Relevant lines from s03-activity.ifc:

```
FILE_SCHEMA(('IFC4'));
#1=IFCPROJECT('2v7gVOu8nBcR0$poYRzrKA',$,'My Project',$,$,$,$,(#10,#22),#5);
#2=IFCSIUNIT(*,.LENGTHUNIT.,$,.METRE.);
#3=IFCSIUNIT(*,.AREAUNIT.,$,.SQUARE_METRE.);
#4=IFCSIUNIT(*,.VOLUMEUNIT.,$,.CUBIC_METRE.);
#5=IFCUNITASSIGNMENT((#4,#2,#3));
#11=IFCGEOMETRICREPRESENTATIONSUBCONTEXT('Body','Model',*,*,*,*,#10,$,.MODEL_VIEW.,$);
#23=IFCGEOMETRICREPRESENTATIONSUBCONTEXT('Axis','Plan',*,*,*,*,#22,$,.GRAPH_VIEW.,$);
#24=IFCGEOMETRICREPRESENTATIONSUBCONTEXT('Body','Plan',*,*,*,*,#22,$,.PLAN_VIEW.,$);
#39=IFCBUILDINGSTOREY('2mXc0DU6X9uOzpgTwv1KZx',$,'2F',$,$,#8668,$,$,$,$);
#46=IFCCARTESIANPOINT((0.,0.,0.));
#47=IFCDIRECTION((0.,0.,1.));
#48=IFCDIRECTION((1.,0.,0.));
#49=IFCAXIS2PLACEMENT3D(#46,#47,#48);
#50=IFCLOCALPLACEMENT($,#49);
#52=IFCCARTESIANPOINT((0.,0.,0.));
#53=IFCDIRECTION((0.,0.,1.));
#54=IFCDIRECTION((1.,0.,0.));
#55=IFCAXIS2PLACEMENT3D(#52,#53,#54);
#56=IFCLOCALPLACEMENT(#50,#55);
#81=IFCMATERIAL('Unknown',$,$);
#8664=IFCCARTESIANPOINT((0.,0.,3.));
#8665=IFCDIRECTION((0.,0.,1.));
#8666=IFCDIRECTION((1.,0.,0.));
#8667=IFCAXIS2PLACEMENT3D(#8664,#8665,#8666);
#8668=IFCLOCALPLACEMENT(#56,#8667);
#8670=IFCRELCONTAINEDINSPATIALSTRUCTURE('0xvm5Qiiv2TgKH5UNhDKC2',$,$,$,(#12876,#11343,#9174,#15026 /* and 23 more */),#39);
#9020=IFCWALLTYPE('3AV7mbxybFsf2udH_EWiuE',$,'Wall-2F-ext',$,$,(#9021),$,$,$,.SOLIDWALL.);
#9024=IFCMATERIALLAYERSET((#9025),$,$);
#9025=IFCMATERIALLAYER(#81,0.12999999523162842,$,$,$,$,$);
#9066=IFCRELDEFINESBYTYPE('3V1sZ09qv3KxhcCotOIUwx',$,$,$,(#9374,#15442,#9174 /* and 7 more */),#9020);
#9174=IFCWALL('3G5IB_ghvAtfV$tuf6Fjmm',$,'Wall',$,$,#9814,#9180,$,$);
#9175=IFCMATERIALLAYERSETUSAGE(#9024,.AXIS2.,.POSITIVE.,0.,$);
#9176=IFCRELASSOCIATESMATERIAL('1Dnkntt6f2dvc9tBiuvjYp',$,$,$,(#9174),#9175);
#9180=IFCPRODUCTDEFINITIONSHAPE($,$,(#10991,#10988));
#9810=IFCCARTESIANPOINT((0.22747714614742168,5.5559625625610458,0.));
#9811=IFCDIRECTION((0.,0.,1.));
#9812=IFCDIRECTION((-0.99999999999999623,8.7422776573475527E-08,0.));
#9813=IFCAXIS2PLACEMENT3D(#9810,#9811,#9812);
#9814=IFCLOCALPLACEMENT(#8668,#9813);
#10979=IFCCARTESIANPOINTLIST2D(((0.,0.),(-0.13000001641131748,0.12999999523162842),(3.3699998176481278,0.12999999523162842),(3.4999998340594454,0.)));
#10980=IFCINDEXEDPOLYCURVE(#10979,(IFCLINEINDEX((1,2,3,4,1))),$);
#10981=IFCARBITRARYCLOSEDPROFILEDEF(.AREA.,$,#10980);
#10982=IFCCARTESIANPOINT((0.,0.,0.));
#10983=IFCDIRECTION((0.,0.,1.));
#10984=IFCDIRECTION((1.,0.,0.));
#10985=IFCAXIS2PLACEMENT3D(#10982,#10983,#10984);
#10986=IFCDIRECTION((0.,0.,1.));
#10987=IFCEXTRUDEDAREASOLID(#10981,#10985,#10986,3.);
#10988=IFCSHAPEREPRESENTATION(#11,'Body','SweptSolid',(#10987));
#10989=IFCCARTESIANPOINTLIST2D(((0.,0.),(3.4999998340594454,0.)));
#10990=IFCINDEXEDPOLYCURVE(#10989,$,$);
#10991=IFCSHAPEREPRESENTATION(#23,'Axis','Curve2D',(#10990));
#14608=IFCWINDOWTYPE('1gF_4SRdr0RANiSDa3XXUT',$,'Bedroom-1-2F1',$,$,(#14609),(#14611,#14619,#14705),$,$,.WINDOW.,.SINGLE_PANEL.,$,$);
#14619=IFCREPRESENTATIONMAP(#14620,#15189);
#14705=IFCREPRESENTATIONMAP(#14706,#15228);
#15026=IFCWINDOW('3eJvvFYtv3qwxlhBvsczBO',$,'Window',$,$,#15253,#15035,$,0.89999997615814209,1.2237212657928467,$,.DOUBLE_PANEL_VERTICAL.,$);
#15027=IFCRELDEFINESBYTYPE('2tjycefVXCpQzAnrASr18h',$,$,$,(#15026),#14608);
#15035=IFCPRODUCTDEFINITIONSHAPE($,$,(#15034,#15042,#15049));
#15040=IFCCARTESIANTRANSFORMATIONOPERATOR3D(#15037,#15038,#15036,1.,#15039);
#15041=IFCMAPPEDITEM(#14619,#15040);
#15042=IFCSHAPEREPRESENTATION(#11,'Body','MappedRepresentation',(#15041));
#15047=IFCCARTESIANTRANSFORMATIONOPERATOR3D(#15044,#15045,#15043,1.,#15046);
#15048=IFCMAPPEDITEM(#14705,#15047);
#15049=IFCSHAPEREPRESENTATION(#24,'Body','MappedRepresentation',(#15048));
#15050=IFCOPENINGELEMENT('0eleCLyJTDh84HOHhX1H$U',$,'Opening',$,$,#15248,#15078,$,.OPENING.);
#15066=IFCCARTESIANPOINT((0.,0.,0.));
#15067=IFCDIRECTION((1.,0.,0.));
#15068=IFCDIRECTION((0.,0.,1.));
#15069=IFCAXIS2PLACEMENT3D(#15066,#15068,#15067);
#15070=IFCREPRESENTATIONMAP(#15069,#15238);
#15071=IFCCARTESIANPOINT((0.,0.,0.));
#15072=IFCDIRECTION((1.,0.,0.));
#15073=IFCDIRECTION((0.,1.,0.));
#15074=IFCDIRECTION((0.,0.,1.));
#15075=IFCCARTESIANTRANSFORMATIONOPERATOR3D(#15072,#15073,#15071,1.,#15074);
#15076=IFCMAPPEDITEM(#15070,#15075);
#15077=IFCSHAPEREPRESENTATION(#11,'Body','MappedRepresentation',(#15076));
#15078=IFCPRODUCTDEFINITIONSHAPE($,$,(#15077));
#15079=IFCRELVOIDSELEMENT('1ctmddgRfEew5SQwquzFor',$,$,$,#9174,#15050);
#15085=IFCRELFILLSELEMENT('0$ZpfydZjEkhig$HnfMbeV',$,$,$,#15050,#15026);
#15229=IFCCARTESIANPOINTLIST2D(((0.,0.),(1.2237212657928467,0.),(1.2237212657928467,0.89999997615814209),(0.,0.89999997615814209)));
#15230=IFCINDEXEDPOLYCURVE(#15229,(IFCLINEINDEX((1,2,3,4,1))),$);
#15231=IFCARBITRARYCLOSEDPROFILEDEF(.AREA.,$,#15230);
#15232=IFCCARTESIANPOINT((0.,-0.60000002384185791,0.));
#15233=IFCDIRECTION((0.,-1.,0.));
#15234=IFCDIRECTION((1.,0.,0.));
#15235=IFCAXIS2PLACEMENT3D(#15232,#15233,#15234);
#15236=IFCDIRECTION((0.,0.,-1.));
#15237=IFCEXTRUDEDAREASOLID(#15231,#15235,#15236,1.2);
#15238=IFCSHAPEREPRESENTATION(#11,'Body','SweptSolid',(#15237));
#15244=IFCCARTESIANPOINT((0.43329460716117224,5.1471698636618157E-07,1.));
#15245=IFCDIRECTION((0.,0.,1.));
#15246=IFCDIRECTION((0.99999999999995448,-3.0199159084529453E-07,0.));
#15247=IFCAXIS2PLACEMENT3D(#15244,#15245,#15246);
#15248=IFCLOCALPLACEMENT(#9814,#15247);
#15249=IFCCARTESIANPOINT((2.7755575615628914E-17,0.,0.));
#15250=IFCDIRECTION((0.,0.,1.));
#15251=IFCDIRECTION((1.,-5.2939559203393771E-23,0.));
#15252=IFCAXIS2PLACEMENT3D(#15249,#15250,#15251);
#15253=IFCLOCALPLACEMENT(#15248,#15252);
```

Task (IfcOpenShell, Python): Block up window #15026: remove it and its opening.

```python
import ifcopenshell
import ifcopenshell.api.feature
import ifcopenshell.api.root
import ifcopenshell.geom
import ifcopenshell.util.shape

model = ifcopenshell.open("s03-activity.ifc")
settings = ifcopenshell.geom.settings()


def volume(element):
    """Net volume in cubic metres, openings subtracted."""
    shape = ifcopenshell.geom.create_shape(settings, element)
    return ifcopenshell.util.shape.get_volume(shape.geometry)


window = model.by_id(15026)
opening = window.FillsVoids[0].RelatingOpeningElement
wall = opening.VoidsElements[0].RelatingBuildingElement
before = volume(wall)

ifcopenshell.api.root.remove_product(model, product=window)
ifcopenshell.api.feature.remove_feature(model, feature=opening)

after = volume(wall)

print(f"wall volume {before:.3f} -> {after:.3f} m3")

model.write("s03-activity-out.ifc")
```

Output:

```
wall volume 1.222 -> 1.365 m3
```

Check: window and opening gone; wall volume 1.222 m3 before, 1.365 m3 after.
